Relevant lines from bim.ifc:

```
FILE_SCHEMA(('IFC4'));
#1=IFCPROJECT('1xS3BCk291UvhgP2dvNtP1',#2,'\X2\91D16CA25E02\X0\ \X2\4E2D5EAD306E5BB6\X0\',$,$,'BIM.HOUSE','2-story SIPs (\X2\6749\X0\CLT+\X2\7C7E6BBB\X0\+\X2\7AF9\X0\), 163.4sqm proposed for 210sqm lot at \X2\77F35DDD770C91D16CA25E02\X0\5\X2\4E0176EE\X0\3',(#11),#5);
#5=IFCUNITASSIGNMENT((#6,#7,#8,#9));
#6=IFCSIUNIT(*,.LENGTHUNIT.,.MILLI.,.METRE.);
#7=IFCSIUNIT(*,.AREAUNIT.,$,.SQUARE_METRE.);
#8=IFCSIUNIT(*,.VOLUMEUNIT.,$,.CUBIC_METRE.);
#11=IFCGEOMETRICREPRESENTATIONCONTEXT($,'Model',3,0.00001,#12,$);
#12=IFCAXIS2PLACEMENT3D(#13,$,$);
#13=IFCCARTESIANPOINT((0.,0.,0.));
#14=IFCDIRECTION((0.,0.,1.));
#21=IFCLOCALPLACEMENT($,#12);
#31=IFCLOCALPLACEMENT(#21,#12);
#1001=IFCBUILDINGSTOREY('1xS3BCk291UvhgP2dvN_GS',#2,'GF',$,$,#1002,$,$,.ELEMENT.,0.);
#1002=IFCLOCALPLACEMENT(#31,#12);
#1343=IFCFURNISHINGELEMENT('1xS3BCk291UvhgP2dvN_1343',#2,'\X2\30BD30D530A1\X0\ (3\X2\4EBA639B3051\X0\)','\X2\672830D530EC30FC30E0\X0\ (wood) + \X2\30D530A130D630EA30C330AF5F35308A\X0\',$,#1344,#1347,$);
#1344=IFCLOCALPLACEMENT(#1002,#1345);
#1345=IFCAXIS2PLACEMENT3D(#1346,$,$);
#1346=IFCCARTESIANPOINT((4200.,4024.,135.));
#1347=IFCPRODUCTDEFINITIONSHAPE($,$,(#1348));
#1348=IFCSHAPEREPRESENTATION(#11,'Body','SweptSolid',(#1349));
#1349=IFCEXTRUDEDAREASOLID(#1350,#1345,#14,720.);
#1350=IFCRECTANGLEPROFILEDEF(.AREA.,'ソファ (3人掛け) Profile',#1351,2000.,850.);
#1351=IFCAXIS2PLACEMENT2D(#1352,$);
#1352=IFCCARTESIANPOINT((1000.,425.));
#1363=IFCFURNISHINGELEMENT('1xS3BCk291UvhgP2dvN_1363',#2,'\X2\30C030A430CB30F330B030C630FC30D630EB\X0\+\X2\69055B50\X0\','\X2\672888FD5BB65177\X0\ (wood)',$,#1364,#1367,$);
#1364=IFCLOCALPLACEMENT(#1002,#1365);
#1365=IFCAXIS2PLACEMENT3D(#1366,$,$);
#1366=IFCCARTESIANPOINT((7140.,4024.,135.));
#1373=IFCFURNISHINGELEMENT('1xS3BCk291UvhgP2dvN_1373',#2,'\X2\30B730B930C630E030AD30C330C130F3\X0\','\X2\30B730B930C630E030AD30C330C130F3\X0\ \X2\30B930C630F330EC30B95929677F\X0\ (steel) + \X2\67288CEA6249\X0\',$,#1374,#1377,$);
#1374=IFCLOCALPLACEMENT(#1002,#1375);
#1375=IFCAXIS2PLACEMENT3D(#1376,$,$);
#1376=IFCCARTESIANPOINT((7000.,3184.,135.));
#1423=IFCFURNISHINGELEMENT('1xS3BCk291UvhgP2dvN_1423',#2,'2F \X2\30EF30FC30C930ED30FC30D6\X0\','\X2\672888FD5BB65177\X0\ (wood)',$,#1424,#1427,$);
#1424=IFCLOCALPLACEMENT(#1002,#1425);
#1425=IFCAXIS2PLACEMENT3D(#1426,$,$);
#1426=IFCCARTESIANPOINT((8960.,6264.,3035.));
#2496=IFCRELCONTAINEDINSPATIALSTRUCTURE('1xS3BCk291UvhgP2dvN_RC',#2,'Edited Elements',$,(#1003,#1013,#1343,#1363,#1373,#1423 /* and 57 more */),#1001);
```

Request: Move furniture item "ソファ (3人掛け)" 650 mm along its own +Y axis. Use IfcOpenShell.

```python
import ifcopenshell
import ifcopenshell.api.geometry
import ifcopenshell.util.placement
import ifcopenshell.util.unit

model = ifcopenshell.open("bim.ifc")
unit_scale = ifcopenshell.util.unit.calculate_unit_scale(model)

item = model.by_id(1343)
matrix = ifcopenshell.util.placement.get_local_placement(item.ObjectPlacement)
matrix[:3, 3] += matrix[:3, 1] * 0.65 / unit_scale
ifcopenshell.api.geometry.edit_object_placement(model, product=item, matrix=matrix, is_si=False)

print(ifcopenshell.util.placement.get_local_placement(item.ObjectPlacement).round(3) + 0.0)

model.write("bim-out.ifc")
```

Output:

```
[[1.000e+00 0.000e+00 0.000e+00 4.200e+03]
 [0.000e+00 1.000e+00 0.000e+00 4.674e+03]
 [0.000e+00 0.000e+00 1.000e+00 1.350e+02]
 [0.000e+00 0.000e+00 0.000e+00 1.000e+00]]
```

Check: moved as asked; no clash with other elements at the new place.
